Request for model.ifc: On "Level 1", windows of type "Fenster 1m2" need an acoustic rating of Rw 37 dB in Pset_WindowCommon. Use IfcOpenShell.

First a look at what the model holds.

```python
import ifcopenshell
import ifcopenshell.util.element

model = ifcopenshell.open("model.ifc")
print(model.schema)
storey = next(s for s in model.by_type("IfcBuildingStorey") if s.Name == "Level 1")
windows = [e for e in ifcopenshell.util.element.get_decomposition(storey) if e.is_a("IfcWindow")]
seen = {}
for e in windows:
    element_type = ifcopenshell.util.element.get_type(e)
    key = (element_type.Name if element_type != e and element_type else None, ifcopenshell.util.element.get_pset(e, "Pset_WindowCommon", "AcousticRating"))
    seen[key] = seen.get(key, 0) + 1
for (name, value), count in sorted(seen.items(), key=str):
    print(count, "x", name, "|", value)
```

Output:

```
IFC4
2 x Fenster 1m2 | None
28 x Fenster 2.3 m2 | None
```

```python
import ifcopenshell
import ifcopenshell.api.pset
import ifcopenshell.util.element

model = ifcopenshell.open("model.ifc")

storey = next(s for s in model.by_type("IfcBuildingStorey") if s.Name == "Level 1")
windows = [e for e in ifcopenshell.util.element.get_decomposition(storey) if e.is_a("IfcWindow")]

count = 0
for e in windows:
    element_type = ifcopenshell.util.element.get_type(e)
    if element_type in (None, e) or element_type.Name != "Fenster 1m2":
        continue
    # add_pset returns the element's existing set when there is one.
    pset = ifcopenshell.api.pset.add_pset(model, product=e, name="Pset_WindowCommon")
    ifcopenshell.api.pset.edit_pset(model, pset=pset, properties={"AcousticRating": "Rw 37 dB"})
    count += 1

print(count, "windows updated")

model.write("model_updated.ifc")
```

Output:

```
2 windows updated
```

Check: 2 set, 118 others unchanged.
